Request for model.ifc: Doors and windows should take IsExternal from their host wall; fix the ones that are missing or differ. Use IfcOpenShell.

First a look at what the model holds.

```python
import ifcopenshell
import ifcopenshell.util.element

model = ifcopenshell.open("model.ifc")
print(model.schema)
seen = {}
for e in model.by_type("IfcDoor") + model.by_type("IfcWindow"):
    if not e.FillsVoids:
        continue
    host = e.FillsVoids[0].RelatingOpeningElement.VoidsElements[0].RelatingBuildingElement
    own = ifcopenshell.util.element.get_pset(e, f"Pset_{e.is_a()[3:].removesuffix('StandardCase')}Common", "IsExternal")
    wall = ifcopenshell.util.element.get_pset(host, "Pset_WallCommon", "IsExternal")
    seen[e.is_a(), own, wall] = seen.get((e.is_a(), own, wall), 0) + 1
for (cls, own, wall), count in sorted(seen.items(), key=str):
    print(count, cls, "IsExternal:", own, "| host wall:", wall)
```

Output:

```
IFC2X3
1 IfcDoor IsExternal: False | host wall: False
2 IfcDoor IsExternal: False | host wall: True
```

```python
import ifcopenshell
import ifcopenshell.api.pset
import ifcopenshell.util.element

model = ifcopenshell.open("model.ifc")

count = 0
for ifc_class, pset_name in (("IfcDoor", "Pset_DoorCommon"), ("IfcWindow", "Pset_WindowCommon")):
    for e in model.by_type(ifc_class):
        if not e.FillsVoids:
            continue
        host = e.FillsVoids[0].RelatingOpeningElement.VoidsElements[0].RelatingBuildingElement
        external = ifcopenshell.util.element.get_pset(host, "Pset_WallCommon", "IsExternal")
        if external is None or ifcopenshell.util.element.get_pset(e, pset_name, "IsExternal") == external:
            continue
        pset = ifcopenshell.api.pset.add_pset(model, product=e, name=pset_name)
        ifcopenshell.api.pset.edit_pset(model, pset=pset, properties={"IsExternal": external})
        count += 1

print(count, "updated")

model.write("model_edited.ifc")
```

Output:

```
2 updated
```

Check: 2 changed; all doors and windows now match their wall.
